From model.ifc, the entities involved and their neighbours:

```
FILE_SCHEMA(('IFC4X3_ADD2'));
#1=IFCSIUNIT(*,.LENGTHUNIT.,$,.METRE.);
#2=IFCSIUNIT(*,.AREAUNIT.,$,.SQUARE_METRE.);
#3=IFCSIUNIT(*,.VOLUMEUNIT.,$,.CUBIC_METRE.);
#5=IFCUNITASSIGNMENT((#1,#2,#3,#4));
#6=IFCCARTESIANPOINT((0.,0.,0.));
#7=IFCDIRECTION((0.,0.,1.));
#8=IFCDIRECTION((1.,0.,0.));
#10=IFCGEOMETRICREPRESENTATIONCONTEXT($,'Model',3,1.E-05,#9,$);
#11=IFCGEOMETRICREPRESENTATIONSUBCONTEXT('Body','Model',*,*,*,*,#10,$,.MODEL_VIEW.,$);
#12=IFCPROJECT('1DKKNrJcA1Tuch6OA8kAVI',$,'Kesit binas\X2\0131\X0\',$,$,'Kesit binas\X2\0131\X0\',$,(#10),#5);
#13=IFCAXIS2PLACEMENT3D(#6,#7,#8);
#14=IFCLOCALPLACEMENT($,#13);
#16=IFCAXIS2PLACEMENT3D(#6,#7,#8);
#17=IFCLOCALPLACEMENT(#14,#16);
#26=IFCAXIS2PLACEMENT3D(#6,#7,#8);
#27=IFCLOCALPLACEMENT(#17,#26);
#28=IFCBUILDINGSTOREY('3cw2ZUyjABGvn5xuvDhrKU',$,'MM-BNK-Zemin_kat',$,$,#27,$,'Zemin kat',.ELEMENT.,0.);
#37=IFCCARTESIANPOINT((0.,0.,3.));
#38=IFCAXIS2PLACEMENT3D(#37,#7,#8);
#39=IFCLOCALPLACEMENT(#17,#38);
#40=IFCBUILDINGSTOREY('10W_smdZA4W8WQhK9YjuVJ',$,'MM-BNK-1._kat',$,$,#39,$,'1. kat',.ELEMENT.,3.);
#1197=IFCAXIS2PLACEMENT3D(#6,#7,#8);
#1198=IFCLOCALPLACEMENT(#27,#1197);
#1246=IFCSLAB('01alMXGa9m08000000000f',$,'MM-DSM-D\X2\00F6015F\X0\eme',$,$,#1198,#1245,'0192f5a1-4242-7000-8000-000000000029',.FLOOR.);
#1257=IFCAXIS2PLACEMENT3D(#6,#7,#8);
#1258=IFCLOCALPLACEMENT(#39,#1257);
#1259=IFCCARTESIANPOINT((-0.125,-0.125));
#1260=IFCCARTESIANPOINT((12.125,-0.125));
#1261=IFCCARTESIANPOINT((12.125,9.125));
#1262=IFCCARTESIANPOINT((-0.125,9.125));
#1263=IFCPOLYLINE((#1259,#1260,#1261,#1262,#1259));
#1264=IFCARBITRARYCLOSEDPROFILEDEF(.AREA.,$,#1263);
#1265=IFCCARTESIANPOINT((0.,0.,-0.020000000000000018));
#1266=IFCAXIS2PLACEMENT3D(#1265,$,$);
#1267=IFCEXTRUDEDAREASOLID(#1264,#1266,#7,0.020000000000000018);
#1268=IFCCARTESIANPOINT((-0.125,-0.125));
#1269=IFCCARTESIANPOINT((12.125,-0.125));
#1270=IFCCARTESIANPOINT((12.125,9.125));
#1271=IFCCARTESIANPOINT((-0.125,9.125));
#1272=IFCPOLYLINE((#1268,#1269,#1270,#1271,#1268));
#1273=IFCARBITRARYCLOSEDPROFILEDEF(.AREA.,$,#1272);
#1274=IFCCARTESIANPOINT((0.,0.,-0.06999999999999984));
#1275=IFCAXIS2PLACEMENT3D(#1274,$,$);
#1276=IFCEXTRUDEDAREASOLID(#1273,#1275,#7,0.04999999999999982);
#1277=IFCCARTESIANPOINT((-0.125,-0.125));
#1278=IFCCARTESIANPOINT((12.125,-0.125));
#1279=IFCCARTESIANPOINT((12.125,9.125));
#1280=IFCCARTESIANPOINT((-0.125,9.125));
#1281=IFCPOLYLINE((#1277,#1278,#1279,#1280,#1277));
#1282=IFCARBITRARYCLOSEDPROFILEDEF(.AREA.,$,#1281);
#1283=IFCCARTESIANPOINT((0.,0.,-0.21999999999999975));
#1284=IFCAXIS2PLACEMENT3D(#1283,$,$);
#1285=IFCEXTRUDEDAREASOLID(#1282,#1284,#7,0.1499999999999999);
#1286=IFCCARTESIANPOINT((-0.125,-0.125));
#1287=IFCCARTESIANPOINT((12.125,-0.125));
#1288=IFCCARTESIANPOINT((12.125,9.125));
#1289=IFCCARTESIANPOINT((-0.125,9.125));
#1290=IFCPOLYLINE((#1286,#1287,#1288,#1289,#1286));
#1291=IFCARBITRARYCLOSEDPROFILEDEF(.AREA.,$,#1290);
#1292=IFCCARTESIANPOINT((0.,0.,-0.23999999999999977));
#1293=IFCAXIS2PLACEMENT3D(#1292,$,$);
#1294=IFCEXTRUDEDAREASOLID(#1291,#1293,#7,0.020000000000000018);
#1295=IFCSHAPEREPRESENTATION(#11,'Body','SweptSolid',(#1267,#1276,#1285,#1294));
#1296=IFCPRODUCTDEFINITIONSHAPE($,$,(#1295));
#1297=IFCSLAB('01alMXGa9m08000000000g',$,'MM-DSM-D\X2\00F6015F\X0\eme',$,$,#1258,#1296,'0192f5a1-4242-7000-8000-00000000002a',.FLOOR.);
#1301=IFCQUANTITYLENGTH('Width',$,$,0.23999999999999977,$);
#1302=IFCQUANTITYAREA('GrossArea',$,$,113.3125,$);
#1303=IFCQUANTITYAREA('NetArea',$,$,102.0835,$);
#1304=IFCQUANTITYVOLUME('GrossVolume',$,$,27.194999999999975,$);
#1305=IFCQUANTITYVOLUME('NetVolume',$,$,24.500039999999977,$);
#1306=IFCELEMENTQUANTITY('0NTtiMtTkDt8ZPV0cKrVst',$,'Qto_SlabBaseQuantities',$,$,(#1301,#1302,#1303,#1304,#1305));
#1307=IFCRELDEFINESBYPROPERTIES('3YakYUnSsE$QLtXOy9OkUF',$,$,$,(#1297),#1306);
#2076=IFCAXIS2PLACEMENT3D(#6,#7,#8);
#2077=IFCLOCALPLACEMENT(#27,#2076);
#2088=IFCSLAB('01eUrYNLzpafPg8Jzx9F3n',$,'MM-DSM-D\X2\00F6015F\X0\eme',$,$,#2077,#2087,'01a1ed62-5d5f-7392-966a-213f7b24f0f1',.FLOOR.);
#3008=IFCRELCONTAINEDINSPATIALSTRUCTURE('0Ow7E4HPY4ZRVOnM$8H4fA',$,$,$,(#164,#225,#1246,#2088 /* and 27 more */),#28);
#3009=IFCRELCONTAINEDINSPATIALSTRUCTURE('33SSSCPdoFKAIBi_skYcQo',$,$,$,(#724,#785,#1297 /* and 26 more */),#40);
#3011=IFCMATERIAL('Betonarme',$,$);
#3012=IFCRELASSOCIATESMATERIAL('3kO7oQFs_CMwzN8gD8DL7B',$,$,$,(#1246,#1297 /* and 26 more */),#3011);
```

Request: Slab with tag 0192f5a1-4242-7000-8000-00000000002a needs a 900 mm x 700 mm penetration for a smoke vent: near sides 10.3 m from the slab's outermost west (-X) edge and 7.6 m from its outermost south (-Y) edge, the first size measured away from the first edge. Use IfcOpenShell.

```python
import numpy as np
import ifcopenshell
import ifcopenshell.api.feature
import ifcopenshell.api.geometry
import ifcopenshell.api.pset
import ifcopenshell.api.root
import ifcopenshell.geom
import ifcopenshell.util.element
import ifcopenshell.util.placement
import ifcopenshell.util.representation
import ifcopenshell.util.shape
import ifcopenshell.util.unit

model = ifcopenshell.open("model.ifc")
unit_scale = ifcopenshell.util.unit.calculate_unit_scale(model)
area_scale = ifcopenshell.util.unit.calculate_unit_scale(model, "AREAUNIT")
volume_scale = ifcopenshell.util.unit.calculate_unit_scale(model, "VOLUMEUNIT")
settings = ifcopenshell.geom.settings()


def volume(element):
    """Net volume in cubic metres, openings subtracted."""
    shape = ifcopenshell.geom.create_shape(settings, element)
    return ifcopenshell.util.shape.get_volume(shape.geometry)


slab = model.by_guid("01alMXGa9m08000000000g")
before = volume(slab)

# Extent in the slab's own axes, in metres. The edges named are its -X and -Y sides.
slab_shape = ifcopenshell.geom.create_shape(settings, slab)
vertices = ifcopenshell.util.shape.get_vertices(slab_shape.geometry)
x_min, y_min, bottom = vertices.min(axis=0)
top = vertices[:, 2].max()

opening = ifcopenshell.api.root.create_entity(model, ifc_class="IfcOpeningElement", name="Smoke vent opening", predefined_type="OPENING")
context = ifcopenshell.util.representation.get_context(model, "Model", "Body", "MODEL_VIEW")
width, depth = 0.9, 0.7
outline = [(0.0, 0.0), (width, 0.0), (width, depth), (0.0, depth), (0.0, 0.0)]
# Overshoot both faces by 50 mm so the cut is clean.
shape = ifcopenshell.api.geometry.add_slab_representation(
    model, context=context, depth=top - bottom + 0.1, polyline=outline
)
ifcopenshell.api.geometry.assign_representation(model, product=opening, representation=shape)

matrix = ifcopenshell.util.placement.get_local_placement(slab.ObjectPlacement)
matrix[:, 3] = matrix @ np.append(np.array([x_min + 10.3, y_min + 7.6, bottom - 0.05]) / unit_scale, 1.0)
ifcopenshell.api.geometry.edit_object_placement(model, product=opening, matrix=matrix, is_si=False)
ifcopenshell.api.feature.add_feature(model, feature=opening, element=slab)

after = volume(slab)

# Update the slab's stored quantities.
qto = model.by_id(ifcopenshell.util.element.get_pset(slab, "Qto_SlabBaseQuantities", should_inherit=False)["id"])
ifcopenshell.api.pset.edit_qto(model, qto=qto, properties={
    "NetArea": after / (top - bottom) / area_scale,
    "NetVolume": after / volume_scale,
})

print(f"slab volume {before:.3f} -> {after:.3f} m3")

model.write("model_edited.ifc")
```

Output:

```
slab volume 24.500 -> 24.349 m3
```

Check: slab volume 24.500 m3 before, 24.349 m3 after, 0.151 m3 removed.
